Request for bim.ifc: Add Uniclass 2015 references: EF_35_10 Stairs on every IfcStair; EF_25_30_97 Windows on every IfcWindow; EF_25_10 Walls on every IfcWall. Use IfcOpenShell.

First a look at what the model holds.

```python
import ifcopenshell

model = ifcopenshell.open("bim.ifc")
print(model.schema)
print("classifications:", [c.Name for c in model.by_type("IfcClassification")])
for ifc_class in ("IfcDoor", "IfcRoof", "IfcStair", "IfcWall", "IfcWindow"):
    print(ifc_class, len(model.by_type(ifc_class)))
```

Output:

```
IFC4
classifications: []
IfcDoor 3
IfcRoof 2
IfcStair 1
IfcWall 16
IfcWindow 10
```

```python
import ifcopenshell
import ifcopenshell.api.classification

model = ifcopenshell.open("bim.ifc")

system = ifcopenshell.api.classification.add_classification(model, classification="Uniclass 2015")

codes = {
    "IfcStair": ("EF_35_10", "Stairs"),
    "IfcWindow": ("EF_25_30_97", "Windows"),
    "IfcWall": ("EF_25_10", "Walls"),
}
for ifc_class, (code, name) in codes.items():
    products = model.by_type(ifc_class)
    ifcopenshell.api.classification.add_reference(
        model, products=products, classification=system, identification=code, name=name
    )
    print(code, len(products))

model.write("bim_edited.ifc")
```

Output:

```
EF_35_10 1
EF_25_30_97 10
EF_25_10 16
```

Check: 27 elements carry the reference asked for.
